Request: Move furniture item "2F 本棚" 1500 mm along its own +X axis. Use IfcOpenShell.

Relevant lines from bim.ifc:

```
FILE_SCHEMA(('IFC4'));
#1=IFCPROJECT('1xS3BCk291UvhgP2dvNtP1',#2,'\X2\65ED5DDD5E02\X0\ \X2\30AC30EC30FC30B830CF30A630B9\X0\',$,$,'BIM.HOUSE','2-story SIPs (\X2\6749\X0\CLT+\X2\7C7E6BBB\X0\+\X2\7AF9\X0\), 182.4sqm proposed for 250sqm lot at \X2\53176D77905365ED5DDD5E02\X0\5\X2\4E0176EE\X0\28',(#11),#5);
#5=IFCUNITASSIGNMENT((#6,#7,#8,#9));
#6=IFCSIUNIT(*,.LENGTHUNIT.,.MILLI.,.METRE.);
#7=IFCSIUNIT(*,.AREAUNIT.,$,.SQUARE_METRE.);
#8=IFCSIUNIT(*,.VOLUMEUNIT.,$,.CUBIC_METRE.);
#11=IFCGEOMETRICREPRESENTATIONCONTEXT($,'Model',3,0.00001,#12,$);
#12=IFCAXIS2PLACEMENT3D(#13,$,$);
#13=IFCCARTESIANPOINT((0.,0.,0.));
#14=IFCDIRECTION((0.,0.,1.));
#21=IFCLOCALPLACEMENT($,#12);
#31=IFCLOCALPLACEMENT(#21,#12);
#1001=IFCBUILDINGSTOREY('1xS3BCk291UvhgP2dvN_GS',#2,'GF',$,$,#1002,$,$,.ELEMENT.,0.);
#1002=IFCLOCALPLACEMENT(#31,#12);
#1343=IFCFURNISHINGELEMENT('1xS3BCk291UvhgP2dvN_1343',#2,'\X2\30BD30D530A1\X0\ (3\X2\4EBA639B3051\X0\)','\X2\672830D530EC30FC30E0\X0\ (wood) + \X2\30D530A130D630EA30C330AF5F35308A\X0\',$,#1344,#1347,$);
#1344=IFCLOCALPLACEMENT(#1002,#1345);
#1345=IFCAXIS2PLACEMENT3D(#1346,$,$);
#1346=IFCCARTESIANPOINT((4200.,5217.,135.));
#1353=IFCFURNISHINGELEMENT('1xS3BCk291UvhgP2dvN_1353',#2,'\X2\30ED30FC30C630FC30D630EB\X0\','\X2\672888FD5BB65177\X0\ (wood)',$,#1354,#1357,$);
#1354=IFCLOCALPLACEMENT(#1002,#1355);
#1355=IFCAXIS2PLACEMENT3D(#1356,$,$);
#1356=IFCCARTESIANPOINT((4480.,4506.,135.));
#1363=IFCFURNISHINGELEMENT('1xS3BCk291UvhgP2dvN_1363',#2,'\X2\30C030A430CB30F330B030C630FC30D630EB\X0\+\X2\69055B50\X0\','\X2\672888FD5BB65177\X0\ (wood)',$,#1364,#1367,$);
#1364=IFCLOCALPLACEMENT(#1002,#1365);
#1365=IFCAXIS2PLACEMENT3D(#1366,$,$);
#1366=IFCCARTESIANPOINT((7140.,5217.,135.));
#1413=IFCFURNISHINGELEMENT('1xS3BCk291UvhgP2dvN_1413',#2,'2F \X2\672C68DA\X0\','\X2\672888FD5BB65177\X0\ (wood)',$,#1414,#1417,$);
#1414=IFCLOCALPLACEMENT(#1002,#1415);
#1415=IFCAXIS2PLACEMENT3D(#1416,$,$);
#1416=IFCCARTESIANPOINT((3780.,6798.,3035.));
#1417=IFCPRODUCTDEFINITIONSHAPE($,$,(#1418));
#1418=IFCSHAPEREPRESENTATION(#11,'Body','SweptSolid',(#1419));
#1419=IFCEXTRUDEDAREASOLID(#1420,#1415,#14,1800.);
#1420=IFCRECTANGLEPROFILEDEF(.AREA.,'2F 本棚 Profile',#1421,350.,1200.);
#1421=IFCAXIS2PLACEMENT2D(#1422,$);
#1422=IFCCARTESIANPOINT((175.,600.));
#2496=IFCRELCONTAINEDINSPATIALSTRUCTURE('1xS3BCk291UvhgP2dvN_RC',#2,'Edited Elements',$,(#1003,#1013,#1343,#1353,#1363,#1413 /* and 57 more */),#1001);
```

```python
import ifcopenshell
import ifcopenshell.api.geometry
import ifcopenshell.util.placement
import ifcopenshell.util.unit

model = ifcopenshell.open("bim.ifc")
unit_scale = ifcopenshell.util.unit.calculate_unit_scale(model)

item = model.by_guid("1xS3BCk291UvhgP2dvN_1413")
matrix = ifcopenshell.util.placement.get_local_placement(item.ObjectPlacement)
matrix[:3, 3] += matrix[:3, 0] * 1.5 / unit_scale
ifcopenshell.api.geometry.edit_object_placement(model, product=item, matrix=matrix, is_si=False)

print(ifcopenshell.util.placement.get_local_placement(item.ObjectPlacement).round(3) + 0.0)

model.write("bim_edited.ifc")
```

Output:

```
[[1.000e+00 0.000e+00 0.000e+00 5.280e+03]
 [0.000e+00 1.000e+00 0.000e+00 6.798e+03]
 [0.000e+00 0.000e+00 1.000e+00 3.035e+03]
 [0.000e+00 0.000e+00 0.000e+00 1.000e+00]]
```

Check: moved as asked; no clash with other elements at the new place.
